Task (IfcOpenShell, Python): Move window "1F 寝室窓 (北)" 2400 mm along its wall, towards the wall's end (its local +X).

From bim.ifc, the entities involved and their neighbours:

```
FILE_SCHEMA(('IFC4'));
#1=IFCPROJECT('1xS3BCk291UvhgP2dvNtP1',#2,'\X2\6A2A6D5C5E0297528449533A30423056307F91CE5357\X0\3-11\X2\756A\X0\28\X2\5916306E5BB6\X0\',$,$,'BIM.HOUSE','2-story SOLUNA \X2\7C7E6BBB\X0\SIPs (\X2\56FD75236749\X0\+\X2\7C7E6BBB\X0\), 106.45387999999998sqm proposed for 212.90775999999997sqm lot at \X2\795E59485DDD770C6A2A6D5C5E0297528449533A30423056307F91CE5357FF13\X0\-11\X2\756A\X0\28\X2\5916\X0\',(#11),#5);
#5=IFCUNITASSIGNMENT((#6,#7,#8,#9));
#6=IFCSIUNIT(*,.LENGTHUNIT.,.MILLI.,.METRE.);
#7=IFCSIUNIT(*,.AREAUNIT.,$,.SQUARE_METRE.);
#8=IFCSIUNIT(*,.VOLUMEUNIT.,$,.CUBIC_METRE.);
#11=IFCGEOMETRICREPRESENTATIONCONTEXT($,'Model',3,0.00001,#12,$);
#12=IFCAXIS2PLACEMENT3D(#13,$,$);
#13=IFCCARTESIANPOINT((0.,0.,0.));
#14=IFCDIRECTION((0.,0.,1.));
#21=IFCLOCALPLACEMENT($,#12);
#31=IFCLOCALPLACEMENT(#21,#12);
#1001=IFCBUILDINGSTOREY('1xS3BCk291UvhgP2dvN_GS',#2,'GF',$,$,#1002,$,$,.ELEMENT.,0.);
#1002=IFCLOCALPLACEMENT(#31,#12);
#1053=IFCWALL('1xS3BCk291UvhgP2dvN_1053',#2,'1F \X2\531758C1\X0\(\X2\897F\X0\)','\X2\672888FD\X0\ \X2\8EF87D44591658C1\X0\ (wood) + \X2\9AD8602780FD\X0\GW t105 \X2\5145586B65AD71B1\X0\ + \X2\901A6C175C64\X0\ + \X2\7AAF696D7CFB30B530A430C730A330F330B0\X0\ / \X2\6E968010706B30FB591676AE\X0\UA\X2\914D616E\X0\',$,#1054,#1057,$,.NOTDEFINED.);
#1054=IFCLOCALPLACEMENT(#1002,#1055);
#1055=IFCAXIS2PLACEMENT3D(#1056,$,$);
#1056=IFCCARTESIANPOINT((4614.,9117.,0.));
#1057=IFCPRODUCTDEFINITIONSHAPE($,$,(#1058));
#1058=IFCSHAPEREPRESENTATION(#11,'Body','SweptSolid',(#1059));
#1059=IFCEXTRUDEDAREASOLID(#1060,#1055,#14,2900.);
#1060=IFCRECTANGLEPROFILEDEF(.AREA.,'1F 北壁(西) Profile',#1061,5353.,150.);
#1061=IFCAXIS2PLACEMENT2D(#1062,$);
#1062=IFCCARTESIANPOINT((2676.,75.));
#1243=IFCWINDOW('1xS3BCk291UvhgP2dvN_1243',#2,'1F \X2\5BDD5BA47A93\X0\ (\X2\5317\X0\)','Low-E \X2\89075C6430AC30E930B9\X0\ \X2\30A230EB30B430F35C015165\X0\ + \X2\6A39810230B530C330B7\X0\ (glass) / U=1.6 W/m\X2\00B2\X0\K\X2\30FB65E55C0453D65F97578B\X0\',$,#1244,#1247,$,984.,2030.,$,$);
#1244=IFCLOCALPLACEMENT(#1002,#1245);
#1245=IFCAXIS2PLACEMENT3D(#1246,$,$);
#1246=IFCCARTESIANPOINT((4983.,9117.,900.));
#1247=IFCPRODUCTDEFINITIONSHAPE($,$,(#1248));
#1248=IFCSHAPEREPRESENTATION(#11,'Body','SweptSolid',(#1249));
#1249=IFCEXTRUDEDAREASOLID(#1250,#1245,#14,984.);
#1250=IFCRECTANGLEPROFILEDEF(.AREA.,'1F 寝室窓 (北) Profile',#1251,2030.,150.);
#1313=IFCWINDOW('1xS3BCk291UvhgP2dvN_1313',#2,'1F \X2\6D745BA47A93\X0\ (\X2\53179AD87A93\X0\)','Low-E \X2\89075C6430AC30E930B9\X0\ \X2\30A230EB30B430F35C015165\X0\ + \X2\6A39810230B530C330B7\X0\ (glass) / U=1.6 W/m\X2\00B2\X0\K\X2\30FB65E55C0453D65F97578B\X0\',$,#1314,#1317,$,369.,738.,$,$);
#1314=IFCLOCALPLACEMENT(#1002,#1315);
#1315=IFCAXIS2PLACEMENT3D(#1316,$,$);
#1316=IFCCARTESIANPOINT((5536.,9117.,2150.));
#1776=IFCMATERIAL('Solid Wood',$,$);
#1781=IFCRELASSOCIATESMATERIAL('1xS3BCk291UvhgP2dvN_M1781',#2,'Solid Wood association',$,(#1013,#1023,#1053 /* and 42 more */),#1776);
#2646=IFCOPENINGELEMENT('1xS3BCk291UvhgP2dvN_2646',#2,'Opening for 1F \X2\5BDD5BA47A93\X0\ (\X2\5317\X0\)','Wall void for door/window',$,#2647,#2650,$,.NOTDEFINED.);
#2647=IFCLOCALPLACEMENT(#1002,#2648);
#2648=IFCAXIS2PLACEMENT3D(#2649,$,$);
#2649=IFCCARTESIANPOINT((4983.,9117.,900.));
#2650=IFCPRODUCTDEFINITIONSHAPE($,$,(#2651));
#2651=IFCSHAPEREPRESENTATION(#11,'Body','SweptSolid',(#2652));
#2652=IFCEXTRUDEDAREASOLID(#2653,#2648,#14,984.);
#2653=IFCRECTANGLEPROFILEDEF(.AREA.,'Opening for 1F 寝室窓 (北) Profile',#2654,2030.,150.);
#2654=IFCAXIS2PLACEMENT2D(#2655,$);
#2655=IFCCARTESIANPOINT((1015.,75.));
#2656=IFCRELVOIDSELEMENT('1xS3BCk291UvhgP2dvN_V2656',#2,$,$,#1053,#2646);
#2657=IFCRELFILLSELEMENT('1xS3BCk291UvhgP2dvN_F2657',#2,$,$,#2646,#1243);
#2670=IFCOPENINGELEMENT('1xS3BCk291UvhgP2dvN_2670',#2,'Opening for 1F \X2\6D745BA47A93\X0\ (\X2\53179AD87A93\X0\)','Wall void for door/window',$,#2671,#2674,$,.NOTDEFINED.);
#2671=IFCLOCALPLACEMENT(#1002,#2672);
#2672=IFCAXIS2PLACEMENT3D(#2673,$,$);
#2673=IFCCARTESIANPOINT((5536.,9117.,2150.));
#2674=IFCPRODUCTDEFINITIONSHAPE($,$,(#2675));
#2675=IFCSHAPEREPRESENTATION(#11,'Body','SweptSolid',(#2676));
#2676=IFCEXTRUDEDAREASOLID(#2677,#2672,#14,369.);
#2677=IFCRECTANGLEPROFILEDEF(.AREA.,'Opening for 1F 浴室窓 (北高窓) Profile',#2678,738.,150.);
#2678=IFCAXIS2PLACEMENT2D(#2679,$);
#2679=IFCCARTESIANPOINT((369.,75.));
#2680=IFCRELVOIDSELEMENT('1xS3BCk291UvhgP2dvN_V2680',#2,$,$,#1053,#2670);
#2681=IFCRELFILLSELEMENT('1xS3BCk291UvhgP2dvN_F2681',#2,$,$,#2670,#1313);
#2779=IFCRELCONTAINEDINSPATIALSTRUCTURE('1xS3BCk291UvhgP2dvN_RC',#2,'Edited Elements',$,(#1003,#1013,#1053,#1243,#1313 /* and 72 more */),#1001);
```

```python
import ifcopenshell
import ifcopenshell.api.geometry
import ifcopenshell.util.placement

model = ifcopenshell.open("bim.ifc")

window = model.by_guid("1xS3BCk291UvhgP2dvN_1243")
opening = window.FillsVoids[0].RelatingOpeningElement
wall = opening.VoidsElements[0].RelatingBuildingElement

wall_matrix = ifcopenshell.util.placement.get_local_placement(wall.ObjectPlacement)
shift = wall_matrix[:3, 0] * 2400.0
before = ifcopenshell.util.placement.get_local_placement(window.ObjectPlacement)[:3, 3].copy()

# The window is not placed relative to its opening, so move both.
for product in (opening, window):
    matrix = ifcopenshell.util.placement.get_local_placement(product.ObjectPlacement)
    matrix[:3, 3] += shift
    ifcopenshell.api.geometry.edit_object_placement(model, product=product, matrix=matrix, is_si=False)

after = ifcopenshell.util.placement.get_local_placement(window.ObjectPlacement)[:3, 3]
print("window moved by", (after - before).round(3) + 0.0)

model.write("bim_v2.ifc")
```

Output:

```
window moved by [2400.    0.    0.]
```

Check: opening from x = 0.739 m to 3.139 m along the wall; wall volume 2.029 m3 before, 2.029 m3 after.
